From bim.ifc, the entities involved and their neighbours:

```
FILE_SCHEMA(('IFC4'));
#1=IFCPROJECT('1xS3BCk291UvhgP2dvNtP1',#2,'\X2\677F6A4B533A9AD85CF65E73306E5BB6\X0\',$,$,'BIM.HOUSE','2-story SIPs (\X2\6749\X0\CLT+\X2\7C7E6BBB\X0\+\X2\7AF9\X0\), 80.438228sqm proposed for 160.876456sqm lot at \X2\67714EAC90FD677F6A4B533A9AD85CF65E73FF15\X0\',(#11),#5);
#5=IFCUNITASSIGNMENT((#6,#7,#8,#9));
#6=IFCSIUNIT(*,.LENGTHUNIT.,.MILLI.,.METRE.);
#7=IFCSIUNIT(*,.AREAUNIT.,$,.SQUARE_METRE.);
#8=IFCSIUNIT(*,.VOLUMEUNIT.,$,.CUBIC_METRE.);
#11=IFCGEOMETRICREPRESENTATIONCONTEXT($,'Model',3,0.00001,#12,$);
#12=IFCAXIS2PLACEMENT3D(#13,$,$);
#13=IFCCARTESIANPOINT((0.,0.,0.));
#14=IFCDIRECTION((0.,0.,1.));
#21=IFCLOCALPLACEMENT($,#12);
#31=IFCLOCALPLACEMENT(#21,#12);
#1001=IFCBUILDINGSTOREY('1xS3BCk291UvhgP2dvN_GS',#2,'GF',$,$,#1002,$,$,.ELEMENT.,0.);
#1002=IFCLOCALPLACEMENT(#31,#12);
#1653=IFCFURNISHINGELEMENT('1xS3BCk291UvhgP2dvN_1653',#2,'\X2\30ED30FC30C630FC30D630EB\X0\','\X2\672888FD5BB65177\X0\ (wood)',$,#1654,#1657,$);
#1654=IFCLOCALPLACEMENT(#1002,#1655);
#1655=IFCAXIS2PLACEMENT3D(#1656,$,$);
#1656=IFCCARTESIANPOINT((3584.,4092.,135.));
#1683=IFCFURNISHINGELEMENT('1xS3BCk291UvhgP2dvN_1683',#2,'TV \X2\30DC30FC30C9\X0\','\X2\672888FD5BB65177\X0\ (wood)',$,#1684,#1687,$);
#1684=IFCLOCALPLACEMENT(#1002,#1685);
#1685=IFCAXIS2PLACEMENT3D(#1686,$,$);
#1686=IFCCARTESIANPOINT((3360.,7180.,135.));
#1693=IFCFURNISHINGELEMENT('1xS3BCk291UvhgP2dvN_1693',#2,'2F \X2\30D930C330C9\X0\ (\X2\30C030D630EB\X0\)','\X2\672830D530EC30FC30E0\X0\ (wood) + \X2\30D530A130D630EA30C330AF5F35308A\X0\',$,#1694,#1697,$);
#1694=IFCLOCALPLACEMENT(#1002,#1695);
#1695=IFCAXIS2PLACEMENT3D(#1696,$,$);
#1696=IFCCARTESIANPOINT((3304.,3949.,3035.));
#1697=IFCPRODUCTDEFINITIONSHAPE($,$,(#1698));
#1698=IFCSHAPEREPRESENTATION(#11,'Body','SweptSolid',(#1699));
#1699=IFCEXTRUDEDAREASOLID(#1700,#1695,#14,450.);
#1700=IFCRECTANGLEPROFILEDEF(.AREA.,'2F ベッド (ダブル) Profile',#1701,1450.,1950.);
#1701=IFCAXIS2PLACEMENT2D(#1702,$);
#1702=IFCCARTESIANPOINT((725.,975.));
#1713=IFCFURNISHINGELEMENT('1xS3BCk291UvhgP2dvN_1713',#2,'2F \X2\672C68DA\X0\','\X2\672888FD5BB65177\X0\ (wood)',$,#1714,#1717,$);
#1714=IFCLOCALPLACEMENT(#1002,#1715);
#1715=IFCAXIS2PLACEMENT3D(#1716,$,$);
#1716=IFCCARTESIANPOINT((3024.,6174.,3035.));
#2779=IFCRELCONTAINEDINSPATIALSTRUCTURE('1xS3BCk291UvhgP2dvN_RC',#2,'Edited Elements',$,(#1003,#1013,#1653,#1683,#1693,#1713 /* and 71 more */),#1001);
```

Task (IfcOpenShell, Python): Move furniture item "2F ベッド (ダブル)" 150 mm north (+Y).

```python
import ifcopenshell
import ifcopenshell.api.geometry
import ifcopenshell.util.placement

model = ifcopenshell.open("bim.ifc")

item = model.by_guid("1xS3BCk291UvhgP2dvN_1693")
matrix = ifcopenshell.util.placement.get_local_placement(item.ObjectPlacement)
matrix[1, 3] += 150.0
ifcopenshell.api.geometry.edit_object_placement(model, product=item, matrix=matrix, is_si=False)

print(ifcopenshell.util.placement.get_local_placement(item.ObjectPlacement).round(3) + 0.0)

model.write("bim_updated.ifc")
```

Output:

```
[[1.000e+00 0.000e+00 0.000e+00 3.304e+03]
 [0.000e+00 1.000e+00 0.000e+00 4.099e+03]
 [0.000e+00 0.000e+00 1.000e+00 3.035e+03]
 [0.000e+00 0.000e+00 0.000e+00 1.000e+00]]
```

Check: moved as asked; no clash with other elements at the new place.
